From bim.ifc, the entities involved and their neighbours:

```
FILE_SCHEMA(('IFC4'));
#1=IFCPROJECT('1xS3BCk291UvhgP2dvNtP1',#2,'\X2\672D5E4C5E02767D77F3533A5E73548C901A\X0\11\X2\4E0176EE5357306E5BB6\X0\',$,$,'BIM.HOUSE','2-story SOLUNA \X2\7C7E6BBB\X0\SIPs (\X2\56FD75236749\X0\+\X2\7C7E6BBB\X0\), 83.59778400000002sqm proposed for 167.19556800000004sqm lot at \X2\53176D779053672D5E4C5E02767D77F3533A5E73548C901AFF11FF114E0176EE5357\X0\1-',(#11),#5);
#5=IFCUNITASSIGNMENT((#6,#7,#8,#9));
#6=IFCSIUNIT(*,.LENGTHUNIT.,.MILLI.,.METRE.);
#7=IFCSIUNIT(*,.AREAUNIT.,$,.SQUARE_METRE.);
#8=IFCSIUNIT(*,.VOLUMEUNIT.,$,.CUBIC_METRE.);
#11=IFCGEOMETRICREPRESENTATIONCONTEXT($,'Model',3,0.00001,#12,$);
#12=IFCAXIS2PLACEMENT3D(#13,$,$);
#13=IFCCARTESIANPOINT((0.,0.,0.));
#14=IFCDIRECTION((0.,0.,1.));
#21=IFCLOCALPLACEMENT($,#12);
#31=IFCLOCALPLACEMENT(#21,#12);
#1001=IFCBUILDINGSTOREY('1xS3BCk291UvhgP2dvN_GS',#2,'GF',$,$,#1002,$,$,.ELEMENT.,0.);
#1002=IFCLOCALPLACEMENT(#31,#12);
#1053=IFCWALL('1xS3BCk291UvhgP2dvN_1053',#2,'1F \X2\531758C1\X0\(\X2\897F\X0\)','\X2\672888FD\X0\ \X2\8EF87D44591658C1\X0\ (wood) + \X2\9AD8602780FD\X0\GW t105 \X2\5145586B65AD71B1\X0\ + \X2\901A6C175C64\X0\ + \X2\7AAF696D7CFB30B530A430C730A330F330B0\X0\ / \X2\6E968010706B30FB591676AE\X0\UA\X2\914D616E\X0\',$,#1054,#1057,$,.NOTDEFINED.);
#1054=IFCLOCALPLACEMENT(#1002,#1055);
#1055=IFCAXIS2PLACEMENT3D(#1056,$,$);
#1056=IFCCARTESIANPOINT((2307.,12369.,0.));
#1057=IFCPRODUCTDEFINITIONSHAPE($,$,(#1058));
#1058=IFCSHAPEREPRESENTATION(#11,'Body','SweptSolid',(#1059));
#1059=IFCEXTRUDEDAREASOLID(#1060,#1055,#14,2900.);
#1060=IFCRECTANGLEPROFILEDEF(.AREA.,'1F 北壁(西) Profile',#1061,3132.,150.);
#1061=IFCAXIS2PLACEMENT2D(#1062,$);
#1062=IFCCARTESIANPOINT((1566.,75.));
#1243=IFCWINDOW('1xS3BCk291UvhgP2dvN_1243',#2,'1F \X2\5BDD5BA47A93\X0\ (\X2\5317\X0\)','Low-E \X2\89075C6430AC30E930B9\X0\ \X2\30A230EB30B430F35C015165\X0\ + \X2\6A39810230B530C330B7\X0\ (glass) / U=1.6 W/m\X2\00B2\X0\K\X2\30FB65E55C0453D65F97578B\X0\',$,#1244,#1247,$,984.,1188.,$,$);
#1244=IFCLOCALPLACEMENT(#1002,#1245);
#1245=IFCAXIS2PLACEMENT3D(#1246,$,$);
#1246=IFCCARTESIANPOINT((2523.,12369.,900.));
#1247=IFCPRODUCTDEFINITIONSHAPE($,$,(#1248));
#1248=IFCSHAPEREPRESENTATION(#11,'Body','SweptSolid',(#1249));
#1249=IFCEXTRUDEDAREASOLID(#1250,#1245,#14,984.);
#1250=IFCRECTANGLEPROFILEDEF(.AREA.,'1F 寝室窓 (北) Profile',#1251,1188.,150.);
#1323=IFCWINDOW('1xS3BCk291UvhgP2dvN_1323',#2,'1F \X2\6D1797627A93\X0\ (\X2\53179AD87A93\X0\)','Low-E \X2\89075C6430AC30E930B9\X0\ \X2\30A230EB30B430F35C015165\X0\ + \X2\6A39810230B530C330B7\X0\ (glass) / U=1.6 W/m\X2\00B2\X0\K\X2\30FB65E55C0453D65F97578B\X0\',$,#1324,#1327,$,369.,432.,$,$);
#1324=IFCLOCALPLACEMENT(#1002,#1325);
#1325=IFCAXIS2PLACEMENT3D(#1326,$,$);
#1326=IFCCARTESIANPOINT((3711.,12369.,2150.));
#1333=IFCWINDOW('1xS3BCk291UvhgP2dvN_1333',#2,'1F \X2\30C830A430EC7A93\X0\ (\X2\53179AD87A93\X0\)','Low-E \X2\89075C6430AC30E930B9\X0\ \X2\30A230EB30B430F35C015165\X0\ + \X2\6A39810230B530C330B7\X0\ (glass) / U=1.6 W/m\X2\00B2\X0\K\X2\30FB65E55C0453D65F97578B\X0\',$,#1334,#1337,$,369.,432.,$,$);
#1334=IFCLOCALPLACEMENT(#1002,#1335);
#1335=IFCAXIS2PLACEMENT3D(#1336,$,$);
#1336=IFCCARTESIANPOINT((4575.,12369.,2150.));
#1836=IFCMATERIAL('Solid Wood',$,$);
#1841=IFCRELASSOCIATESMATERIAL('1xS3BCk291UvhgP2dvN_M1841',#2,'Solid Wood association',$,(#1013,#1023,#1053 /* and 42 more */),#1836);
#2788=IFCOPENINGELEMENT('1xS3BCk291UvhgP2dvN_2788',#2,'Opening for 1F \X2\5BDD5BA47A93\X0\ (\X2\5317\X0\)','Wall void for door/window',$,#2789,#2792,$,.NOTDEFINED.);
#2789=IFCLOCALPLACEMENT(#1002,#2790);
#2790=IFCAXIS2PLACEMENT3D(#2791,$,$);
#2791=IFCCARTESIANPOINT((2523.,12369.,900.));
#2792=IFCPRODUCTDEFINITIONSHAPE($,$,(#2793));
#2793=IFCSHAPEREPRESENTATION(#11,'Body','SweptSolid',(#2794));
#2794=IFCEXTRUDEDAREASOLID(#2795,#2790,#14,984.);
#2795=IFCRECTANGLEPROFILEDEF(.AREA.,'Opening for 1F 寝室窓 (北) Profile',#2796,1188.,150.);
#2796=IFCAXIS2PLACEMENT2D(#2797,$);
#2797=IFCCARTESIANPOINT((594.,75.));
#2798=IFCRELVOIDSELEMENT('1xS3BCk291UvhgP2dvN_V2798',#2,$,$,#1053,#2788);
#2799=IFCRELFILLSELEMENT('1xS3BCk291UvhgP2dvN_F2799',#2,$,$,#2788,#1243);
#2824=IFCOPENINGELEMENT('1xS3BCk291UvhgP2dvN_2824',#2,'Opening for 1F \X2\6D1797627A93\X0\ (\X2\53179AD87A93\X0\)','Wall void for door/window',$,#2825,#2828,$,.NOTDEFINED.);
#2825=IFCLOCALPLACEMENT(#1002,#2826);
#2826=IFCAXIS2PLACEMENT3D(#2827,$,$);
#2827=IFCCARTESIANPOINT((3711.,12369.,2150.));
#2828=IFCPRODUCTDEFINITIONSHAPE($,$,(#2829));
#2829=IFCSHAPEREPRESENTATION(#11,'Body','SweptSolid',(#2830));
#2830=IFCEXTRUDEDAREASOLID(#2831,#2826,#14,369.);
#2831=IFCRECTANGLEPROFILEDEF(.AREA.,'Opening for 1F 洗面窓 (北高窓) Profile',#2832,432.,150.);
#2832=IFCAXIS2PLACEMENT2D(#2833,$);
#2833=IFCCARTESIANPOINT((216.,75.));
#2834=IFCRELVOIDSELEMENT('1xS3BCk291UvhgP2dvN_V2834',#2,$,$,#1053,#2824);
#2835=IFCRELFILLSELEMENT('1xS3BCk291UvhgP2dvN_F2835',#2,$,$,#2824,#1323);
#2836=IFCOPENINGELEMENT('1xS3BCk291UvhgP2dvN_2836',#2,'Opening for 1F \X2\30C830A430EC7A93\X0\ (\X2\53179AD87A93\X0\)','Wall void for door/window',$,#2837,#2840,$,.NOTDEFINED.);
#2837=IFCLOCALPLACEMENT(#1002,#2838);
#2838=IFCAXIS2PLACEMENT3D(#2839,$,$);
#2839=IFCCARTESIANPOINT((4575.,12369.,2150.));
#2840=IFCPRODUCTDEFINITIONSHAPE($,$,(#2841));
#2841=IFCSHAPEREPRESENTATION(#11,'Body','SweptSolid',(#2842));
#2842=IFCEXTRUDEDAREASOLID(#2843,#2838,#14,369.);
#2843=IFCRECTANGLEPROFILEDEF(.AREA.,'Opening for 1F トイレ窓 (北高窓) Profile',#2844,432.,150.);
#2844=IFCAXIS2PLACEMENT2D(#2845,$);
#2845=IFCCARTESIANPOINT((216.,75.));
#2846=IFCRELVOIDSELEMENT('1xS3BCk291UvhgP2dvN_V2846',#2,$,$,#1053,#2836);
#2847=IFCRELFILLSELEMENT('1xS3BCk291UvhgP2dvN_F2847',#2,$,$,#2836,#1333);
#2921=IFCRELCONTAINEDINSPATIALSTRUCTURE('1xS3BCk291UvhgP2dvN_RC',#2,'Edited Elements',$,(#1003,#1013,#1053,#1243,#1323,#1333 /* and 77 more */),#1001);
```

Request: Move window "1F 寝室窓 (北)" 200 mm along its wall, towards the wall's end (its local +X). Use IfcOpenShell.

```python
import ifcopenshell
import ifcopenshell.api.geometry
import ifcopenshell.util.placement

model = ifcopenshell.open("bim.ifc")

window = model.by_guid("1xS3BCk291UvhgP2dvN_1243")
opening = window.FillsVoids[0].RelatingOpeningElement
wall = opening.VoidsElements[0].RelatingBuildingElement

wall_matrix = ifcopenshell.util.placement.get_local_placement(wall.ObjectPlacement)
shift = wall_matrix[:3, 0] * 200.0
before = ifcopenshell.util.placement.get_local_placement(window.ObjectPlacement)[:3, 3].copy()

# The window is not placed relative to its opening, so move both.
for product in (opening, window):
    matrix = ifcopenshell.util.placement.get_local_placement(product.ObjectPlacement)
    matrix[:3, 3] += shift
    ifcopenshell.api.geometry.edit_object_placement(model, product=product, matrix=matrix, is_si=False)

after = ifcopenshell.util.placement.get_local_placement(window.ObjectPlacement)[:3, 3]
print("window moved by", (after - before).round(3) + 0.0)

model.write("bim_rev.ifc")
```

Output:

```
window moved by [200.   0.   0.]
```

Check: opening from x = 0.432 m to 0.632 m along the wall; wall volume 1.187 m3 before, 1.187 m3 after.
